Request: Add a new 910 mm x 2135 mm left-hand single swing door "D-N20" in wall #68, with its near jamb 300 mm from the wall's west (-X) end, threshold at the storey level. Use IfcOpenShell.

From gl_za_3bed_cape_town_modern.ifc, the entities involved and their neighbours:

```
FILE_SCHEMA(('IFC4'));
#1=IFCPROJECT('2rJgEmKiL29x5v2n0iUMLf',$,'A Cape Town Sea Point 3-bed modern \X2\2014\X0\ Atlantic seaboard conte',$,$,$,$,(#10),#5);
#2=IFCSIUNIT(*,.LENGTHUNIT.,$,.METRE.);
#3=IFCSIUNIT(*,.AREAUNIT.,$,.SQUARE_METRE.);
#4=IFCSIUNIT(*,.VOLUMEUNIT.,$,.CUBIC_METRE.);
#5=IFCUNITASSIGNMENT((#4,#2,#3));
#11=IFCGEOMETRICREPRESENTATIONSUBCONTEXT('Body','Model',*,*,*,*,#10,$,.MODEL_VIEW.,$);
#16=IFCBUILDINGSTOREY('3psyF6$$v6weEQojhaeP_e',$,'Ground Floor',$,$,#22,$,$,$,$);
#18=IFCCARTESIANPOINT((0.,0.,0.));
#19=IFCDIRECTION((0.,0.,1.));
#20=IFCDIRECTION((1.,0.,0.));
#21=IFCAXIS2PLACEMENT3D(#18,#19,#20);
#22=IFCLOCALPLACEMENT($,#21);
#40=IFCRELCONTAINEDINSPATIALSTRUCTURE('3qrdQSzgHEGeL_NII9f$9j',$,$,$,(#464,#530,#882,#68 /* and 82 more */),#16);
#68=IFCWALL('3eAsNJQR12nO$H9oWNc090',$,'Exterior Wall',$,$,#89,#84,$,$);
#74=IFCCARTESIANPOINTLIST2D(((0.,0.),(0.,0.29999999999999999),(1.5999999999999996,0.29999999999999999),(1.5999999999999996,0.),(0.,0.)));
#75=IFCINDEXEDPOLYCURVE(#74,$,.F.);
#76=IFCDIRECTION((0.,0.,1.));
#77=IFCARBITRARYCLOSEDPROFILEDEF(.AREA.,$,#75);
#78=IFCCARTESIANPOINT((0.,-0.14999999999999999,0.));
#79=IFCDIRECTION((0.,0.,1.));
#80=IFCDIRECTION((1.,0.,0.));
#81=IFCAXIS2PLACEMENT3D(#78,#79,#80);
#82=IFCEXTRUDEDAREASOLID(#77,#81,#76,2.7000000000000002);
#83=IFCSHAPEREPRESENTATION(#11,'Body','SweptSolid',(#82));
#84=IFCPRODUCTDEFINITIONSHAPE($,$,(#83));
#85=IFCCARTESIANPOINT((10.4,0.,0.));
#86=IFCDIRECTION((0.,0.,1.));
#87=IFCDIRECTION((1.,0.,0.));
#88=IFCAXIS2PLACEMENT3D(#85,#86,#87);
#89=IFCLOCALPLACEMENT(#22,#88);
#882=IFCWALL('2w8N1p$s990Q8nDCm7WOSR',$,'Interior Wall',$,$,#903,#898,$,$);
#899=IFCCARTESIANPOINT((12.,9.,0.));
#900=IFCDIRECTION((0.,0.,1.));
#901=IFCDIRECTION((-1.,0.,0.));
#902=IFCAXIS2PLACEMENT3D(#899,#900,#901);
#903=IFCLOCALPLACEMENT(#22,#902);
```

```python
import numpy as np
import ifcopenshell
import ifcopenshell.api.feature
import ifcopenshell.api.geometry
import ifcopenshell.api.root
import ifcopenshell.api.spatial
import ifcopenshell.geom
import ifcopenshell.util.element
import ifcopenshell.util.placement
import ifcopenshell.util.representation
import ifcopenshell.util.shape
import ifcopenshell.util.unit

model = ifcopenshell.open("gl_za_3bed_cape_town_modern.ifc")
unit_scale = ifcopenshell.util.unit.calculate_unit_scale(model)
settings = ifcopenshell.geom.settings()


def volume(element):
    """Net volume in cubic metres, openings subtracted."""
    shape = ifcopenshell.geom.create_shape(settings, element)
    return ifcopenshell.util.shape.get_volume(shape.geometry)


wall = model.by_guid("3eAsNJQR12nO$H9oWNc090")
storey = ifcopenshell.util.element.get_container(wall, ifc_class="IfcBuildingStorey")
context = ifcopenshell.util.representation.get_context(model, "Model", "Body", "MODEL_VIEW")
before = volume(wall)

width, height, from_end, sill = 0.91, 2.135, 0.3, 0.0  # metres

# The wall runs along its own X axis, and the end named is its -X end.
wall_shape = ifcopenshell.geom.create_shape(settings, wall)
x, y, z = ifcopenshell.util.shape.get_vertices(wall_shape.geometry).T
start = x.min() + from_end
face, thickness = float(y.min()), float(y.max() - y.min())
wall_matrix = ifcopenshell.util.placement.get_local_placement(wall.ObjectPlacement)
level = ifcopenshell.util.placement.get_local_placement(storey.ObjectPlacement)[2, 3]


def in_wall(x, y):
    """Placement at x, y metres in the wall's axes, at sill height."""
    matrix = wall_matrix.copy()
    matrix[:, 3] = wall_matrix @ np.array([x / unit_scale, y / unit_scale, 0.0, 1.0])
    matrix[2, 3] = level + sill / unit_scale
    return matrix


# Opening: a box that overshoots both wall faces by 50 mm.
opening = ifcopenshell.api.root.create_entity(model, ifc_class="IfcOpeningElement", predefined_type="OPENING")
box = ifcopenshell.api.geometry.add_wall_representation(
    model, context=context, length=width, height=height, thickness=thickness + 0.1
)
ifcopenshell.api.geometry.assign_representation(model, product=opening, representation=box)
ifcopenshell.api.geometry.edit_object_placement(model, product=opening, matrix=in_wall(start, face - 0.05), is_si=False)
ifcopenshell.api.feature.add_feature(model, feature=opening, element=wall)

door = ifcopenshell.api.root.create_entity(model, ifc_class="IfcDoor", name="D-N20", predefined_type="DOOR")
door.OverallWidth, door.OverallHeight = width / unit_scale, height / unit_scale
door.OperationType = "SINGLE_SWING_LEFT"
body = ifcopenshell.api.geometry.add_door_representation(
    model,
    context=context,
    overall_width=door.OverallWidth,
    overall_height=door.OverallHeight,
    operation_type="SINGLE_SWING_LEFT",
    lining_properties={"LiningDepth": thickness / unit_scale, "ThresholdDepth": thickness / unit_scale},
)
ifcopenshell.api.geometry.assign_representation(model, product=door, representation=body)
ifcopenshell.api.spatial.assign_container(model, products=[door], relating_structure=storey)
ifcopenshell.api.feature.add_filling(model, opening=opening, element=door)

# The lining spans the wall, so the door starts at the wall face.
ifcopenshell.api.geometry.edit_object_placement(model, product=door, matrix=in_wall(start, face), is_si=False)

after = volume(wall)

print(f"wall volume {before:.3f} -> {after:.3f} m3")

model.write("gl_za_3bed_cape_town_modern_v2.ifc")
```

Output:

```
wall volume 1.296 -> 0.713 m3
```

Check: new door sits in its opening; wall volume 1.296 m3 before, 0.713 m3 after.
